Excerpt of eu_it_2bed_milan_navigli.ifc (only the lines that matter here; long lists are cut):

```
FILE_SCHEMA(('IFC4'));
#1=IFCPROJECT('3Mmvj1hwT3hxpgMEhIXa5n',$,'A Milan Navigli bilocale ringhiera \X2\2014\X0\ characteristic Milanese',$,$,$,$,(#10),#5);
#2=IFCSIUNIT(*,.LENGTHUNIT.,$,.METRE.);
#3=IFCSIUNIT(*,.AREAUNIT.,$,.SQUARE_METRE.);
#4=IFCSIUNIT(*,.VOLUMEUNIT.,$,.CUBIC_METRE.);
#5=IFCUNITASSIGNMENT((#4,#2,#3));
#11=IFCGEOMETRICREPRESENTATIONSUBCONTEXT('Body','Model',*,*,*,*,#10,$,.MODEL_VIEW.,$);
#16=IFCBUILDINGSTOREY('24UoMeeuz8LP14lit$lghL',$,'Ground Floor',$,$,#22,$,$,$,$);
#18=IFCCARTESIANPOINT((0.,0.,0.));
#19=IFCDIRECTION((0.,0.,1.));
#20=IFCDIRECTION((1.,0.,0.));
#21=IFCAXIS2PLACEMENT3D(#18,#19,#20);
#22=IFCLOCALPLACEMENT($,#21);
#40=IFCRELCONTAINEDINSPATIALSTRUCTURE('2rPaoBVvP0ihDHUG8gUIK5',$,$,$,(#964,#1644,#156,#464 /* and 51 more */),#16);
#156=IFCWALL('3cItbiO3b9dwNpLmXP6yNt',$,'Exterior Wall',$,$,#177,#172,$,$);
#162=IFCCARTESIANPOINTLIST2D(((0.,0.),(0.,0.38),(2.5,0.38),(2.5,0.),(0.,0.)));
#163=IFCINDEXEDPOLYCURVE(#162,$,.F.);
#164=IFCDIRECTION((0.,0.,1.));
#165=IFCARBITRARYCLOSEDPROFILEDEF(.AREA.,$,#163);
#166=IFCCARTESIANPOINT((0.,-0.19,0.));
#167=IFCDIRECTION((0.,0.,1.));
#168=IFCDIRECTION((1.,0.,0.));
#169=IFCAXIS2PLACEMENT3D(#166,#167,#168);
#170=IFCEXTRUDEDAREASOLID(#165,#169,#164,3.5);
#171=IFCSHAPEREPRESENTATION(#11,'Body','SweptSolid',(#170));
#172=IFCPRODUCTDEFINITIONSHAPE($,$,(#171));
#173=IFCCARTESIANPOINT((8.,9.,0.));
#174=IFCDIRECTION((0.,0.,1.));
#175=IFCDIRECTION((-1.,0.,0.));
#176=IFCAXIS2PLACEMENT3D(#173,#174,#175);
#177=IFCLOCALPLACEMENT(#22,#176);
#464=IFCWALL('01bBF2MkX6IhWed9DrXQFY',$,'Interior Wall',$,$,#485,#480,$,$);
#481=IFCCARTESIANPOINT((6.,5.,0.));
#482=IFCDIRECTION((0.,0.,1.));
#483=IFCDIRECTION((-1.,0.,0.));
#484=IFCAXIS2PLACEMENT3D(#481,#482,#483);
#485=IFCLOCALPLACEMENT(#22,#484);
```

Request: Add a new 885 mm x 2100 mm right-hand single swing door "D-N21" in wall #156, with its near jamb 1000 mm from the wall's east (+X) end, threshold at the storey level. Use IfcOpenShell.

```python
import numpy as np
import ifcopenshell
import ifcopenshell.api.feature
import ifcopenshell.api.geometry
import ifcopenshell.api.root
import ifcopenshell.api.spatial
import ifcopenshell.geom
import ifcopenshell.util.element
import ifcopenshell.util.placement
import ifcopenshell.util.representation
import ifcopenshell.util.shape
import ifcopenshell.util.unit

model = ifcopenshell.open("eu_it_2bed_milan_navigli.ifc")
unit_scale = ifcopenshell.util.unit.calculate_unit_scale(model)
settings = ifcopenshell.geom.settings()


def volume(element):
    """Net volume in cubic metres, openings subtracted."""
    shape = ifcopenshell.geom.create_shape(settings, element)
    return ifcopenshell.util.shape.get_volume(shape.geometry)


wall = model.by_guid("3cItbiO3b9dwNpLmXP6yNt")
storey = ifcopenshell.util.element.get_container(wall, ifc_class="IfcBuildingStorey")
context = ifcopenshell.util.representation.get_context(model, "Model", "Body", "MODEL_VIEW")
before = volume(wall)

width, height, from_end, sill = 0.885, 2.1, 1, 0.0  # metres

# The wall runs along its own X axis, and the end named is its -X end.
wall_shape = ifcopenshell.geom.create_shape(settings, wall)
x, y, z = ifcopenshell.util.shape.get_vertices(wall_shape.geometry).T
start = x.min() + from_end
face, thickness = float(y.min()), float(y.max() - y.min())
wall_matrix = ifcopenshell.util.placement.get_local_placement(wall.ObjectPlacement)
level = ifcopenshell.util.placement.get_local_placement(storey.ObjectPlacement)[2, 3]


def in_wall(x, y):
    """Placement at x, y metres in the wall's axes, at sill height."""
    matrix = wall_matrix.copy()
    matrix[:, 3] = wall_matrix @ np.array([x / unit_scale, y / unit_scale, 0.0, 1.0])
    matrix[2, 3] = level + sill / unit_scale
    return matrix


# Opening: a box that overshoots both wall faces by 50 mm.
opening = ifcopenshell.api.root.create_entity(model, ifc_class="IfcOpeningElement", predefined_type="OPENING")
box = ifcopenshell.api.geometry.add_wall_representation(
    model, context=context, length=width, height=height, thickness=thickness + 0.1
)
ifcopenshell.api.geometry.assign_representation(model, product=opening, representation=box)
ifcopenshell.api.geometry.edit_object_placement(model, product=opening, matrix=in_wall(start, face - 0.05), is_si=False)
ifcopenshell.api.feature.add_feature(model, feature=opening, element=wall)

door = ifcopenshell.api.root.create_entity(model, ifc_class="IfcDoor", name="D-N21", predefined_type="DOOR")
door.OverallWidth, door.OverallHeight = width / unit_scale, height / unit_scale
door.OperationType = "SINGLE_SWING_RIGHT"
body = ifcopenshell.api.geometry.add_door_representation(
    model,
    context=context,
    overall_width=door.OverallWidth,
    overall_height=door.OverallHeight,
    operation_type="SINGLE_SWING_RIGHT",
    lining_properties={"LiningDepth": thickness / unit_scale, "ThresholdDepth": thickness / unit_scale},
)
ifcopenshell.api.geometry.assign_representation(model, product=door, representation=body)
ifcopenshell.api.spatial.assign_container(model, products=[door], relating_structure=storey)
ifcopenshell.api.feature.add_filling(model, opening=opening, element=door)

# The lining spans the wall, so the door starts at the wall face.
ifcopenshell.api.geometry.edit_object_placement(model, product=door, matrix=in_wall(start, face), is_si=False)

after = volume(wall)

print(f"wall volume {before:.3f} -> {after:.3f} m3")

model.write("eu_it_2bed_milan_navigli-out.ifc")
```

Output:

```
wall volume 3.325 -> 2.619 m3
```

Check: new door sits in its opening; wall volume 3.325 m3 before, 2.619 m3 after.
